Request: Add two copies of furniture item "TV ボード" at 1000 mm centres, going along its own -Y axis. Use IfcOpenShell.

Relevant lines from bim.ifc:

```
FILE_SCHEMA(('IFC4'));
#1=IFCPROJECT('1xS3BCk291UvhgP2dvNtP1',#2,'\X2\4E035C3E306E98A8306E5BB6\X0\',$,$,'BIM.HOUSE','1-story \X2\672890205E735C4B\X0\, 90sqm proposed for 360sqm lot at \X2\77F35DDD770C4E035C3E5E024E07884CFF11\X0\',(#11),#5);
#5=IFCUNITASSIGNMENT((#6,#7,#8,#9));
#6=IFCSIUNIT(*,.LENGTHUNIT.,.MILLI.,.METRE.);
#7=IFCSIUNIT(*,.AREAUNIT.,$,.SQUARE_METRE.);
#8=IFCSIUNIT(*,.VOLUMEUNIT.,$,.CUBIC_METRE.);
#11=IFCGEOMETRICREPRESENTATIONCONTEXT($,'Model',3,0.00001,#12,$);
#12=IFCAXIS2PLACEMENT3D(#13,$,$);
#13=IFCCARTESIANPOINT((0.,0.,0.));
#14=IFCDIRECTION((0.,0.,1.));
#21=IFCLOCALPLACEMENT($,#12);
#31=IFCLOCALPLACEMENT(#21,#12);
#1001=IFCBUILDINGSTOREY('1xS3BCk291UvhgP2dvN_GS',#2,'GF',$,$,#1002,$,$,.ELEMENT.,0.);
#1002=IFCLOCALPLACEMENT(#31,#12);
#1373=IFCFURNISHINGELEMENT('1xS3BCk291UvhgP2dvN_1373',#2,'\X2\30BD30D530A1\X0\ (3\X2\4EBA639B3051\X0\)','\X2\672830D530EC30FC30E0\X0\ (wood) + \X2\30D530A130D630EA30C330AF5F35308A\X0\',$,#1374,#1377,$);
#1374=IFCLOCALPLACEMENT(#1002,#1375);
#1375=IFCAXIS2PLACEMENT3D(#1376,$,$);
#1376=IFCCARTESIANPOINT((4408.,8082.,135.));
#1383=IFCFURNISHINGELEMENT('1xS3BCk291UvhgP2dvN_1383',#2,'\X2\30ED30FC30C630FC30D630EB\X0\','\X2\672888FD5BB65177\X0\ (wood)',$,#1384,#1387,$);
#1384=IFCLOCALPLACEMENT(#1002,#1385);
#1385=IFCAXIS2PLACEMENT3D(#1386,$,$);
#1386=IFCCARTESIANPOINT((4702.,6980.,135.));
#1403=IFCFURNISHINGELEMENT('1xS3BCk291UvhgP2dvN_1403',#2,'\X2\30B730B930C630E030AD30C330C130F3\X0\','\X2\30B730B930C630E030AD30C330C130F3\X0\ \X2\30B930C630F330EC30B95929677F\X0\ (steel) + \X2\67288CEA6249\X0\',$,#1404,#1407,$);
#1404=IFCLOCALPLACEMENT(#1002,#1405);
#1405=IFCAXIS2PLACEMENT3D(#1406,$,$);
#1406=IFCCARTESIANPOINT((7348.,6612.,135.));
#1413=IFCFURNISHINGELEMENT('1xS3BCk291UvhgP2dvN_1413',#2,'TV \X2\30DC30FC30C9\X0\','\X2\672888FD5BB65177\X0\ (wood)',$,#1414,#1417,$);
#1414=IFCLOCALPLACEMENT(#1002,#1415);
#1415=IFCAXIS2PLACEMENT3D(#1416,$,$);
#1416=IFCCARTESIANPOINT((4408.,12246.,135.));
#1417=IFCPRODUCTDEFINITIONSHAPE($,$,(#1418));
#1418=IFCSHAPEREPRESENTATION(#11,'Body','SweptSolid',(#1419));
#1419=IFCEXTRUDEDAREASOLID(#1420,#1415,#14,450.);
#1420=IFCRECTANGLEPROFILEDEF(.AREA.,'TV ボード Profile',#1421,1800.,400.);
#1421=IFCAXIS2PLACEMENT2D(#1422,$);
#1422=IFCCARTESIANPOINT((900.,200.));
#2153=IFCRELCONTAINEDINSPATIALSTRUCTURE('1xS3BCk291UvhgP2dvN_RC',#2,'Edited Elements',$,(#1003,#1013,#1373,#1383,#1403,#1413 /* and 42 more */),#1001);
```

```python
import ifcopenshell
import ifcopenshell.api.geometry
import ifcopenshell.api.root
import ifcopenshell.util.element
import ifcopenshell.util.placement

model = ifcopenshell.open("bim.ifc")


def reuse_history(source, copy):
    """copy_class also copies each property set's owner history, people and application; keep the originals."""
    for rel in copy.IsDefinedBy:
        if rel.is_a("IfcRelDefinesByProperties") and (history := rel.RelatingPropertyDefinition.OwnerHistory):
            rel.RelatingPropertyDefinition.OwnerHistory = source.OwnerHistory
            ifcopenshell.util.element.remove_deep2(model, history)


source = model.by_guid("1xS3BCk291UvhgP2dvN_1413")
base = ifcopenshell.util.placement.get_local_placement(source.ObjectPlacement)
step = -base[:3, 1] * 1000.0

for i in range(1, 3):
    copy = ifcopenshell.api.root.copy_class(model, product=source)
    copy.Representation = ifcopenshell.util.element.copy_deep(
        model, source.Representation, exclude=["IfcGeometricRepresentationContext", "IfcRepresentationMap"]
    )
    reuse_history(source, copy)
    matrix = base.copy()
    matrix[:3, 3] += i * step
    print("added at", matrix[:3, 3].round(3) + 0.0)
    ifcopenshell.api.geometry.edit_object_placement(model, product=copy, matrix=matrix, is_si=False)

model.write("bim-out.ifc")
```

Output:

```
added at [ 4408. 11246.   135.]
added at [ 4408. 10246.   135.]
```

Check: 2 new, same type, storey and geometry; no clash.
